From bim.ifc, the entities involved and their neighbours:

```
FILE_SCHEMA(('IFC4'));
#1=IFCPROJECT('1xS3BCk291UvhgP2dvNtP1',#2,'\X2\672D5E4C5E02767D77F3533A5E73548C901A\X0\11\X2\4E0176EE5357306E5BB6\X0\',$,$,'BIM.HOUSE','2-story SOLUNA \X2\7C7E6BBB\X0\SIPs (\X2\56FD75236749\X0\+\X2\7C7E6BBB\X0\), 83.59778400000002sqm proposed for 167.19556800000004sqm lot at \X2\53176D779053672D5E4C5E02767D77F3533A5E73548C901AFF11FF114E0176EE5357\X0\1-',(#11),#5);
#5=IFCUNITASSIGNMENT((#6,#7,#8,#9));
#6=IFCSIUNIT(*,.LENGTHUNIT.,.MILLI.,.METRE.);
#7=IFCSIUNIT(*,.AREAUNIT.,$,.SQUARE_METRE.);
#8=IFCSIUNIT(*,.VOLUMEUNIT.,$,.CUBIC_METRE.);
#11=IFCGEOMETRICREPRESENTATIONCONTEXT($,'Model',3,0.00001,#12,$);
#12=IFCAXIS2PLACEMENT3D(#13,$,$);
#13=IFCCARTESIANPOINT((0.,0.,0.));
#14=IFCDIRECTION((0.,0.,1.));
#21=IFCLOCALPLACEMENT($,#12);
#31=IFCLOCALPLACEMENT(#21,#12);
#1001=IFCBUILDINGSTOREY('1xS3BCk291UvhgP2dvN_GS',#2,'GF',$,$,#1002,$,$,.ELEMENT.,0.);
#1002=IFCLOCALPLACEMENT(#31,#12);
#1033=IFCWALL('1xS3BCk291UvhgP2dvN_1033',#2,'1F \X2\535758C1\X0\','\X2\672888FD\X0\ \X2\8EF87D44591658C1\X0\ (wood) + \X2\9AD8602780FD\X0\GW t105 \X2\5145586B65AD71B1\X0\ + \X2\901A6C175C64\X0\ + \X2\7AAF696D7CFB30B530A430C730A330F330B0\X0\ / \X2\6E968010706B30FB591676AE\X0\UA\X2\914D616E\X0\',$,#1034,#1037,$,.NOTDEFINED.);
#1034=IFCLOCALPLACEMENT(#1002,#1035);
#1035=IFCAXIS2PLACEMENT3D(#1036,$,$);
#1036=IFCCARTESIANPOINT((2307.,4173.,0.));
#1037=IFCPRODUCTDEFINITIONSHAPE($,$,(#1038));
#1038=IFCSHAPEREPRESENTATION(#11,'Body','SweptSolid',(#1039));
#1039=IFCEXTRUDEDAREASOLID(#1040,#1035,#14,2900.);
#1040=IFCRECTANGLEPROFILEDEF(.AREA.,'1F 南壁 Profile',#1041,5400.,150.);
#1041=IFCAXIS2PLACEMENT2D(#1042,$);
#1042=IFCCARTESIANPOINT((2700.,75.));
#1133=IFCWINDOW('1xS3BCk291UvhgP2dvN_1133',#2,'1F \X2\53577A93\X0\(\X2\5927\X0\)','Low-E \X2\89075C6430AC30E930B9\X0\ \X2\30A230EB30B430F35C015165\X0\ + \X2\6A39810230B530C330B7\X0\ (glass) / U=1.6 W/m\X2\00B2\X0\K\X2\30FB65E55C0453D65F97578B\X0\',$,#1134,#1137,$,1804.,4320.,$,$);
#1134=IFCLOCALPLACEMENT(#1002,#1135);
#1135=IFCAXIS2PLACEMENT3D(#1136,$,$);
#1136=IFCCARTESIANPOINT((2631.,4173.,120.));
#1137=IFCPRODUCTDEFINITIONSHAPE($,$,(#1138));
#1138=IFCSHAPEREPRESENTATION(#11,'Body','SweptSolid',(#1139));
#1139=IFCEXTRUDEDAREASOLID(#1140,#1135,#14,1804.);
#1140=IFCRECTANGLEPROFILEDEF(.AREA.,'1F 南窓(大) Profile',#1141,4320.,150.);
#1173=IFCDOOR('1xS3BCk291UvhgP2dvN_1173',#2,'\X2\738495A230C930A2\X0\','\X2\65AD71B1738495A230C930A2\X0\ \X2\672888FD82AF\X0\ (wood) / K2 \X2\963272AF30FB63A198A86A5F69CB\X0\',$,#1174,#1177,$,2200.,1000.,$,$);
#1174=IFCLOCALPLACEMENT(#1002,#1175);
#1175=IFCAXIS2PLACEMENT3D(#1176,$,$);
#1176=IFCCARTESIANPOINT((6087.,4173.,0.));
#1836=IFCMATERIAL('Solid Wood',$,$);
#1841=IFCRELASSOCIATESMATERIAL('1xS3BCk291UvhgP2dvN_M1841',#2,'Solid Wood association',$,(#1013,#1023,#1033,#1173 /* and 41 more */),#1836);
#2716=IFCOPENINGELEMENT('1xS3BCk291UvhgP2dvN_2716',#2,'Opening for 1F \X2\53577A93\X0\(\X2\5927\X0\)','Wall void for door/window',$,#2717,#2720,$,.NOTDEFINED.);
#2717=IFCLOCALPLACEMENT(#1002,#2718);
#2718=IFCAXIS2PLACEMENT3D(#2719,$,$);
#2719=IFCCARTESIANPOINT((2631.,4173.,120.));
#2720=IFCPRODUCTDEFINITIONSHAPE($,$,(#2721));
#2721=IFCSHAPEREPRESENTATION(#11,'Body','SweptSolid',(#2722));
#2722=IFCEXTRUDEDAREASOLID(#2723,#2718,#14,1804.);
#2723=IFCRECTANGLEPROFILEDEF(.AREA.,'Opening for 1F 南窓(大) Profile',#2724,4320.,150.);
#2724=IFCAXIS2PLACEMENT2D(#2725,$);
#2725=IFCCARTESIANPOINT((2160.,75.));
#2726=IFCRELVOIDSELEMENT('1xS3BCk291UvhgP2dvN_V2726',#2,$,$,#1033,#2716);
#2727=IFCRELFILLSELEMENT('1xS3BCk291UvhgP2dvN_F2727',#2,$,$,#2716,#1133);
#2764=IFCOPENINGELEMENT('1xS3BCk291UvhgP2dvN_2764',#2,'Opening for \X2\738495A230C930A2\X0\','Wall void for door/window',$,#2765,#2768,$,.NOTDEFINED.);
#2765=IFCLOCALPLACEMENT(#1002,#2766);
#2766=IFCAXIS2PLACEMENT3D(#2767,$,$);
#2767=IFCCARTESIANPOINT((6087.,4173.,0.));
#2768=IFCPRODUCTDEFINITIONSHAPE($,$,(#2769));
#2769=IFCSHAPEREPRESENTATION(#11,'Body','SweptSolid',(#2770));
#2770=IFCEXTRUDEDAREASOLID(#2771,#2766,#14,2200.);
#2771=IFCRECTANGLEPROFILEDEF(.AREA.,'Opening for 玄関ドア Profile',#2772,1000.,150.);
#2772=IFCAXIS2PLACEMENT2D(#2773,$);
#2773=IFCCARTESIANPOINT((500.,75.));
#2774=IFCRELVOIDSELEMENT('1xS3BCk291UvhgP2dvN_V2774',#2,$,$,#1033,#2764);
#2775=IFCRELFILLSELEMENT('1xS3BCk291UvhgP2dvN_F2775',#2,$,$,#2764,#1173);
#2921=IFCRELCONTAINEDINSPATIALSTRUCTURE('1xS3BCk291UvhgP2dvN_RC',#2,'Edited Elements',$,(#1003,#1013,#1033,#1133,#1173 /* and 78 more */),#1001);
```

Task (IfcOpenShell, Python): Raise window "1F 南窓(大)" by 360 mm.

```python
import numpy as np
import ifcopenshell
import ifcopenshell.api.geometry
import ifcopenshell.util.placement
import ifcopenshell.util.unit

model = ifcopenshell.open("bim.ifc")
unit_scale = ifcopenshell.util.unit.calculate_unit_scale(model)

window = model.by_guid("1xS3BCk291UvhgP2dvN_1133")
opening = window.FillsVoids[0].RelatingOpeningElement
dz = 0.36 / unit_scale

shift = np.array([0.0, 0.0, dz])
# The window is not placed relative to its opening, so move both.
for product in (opening, window):
    matrix = ifcopenshell.util.placement.get_local_placement(product.ObjectPlacement)
    matrix[:3, 3] += shift
    ifcopenshell.api.geometry.edit_object_placement(model, product=product, matrix=matrix, is_si=False)

print(f"moved by {dz * unit_scale:+.3f} m")

model.write("bim-out.ifc")
```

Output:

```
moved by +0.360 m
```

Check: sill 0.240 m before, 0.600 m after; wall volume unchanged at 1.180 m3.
